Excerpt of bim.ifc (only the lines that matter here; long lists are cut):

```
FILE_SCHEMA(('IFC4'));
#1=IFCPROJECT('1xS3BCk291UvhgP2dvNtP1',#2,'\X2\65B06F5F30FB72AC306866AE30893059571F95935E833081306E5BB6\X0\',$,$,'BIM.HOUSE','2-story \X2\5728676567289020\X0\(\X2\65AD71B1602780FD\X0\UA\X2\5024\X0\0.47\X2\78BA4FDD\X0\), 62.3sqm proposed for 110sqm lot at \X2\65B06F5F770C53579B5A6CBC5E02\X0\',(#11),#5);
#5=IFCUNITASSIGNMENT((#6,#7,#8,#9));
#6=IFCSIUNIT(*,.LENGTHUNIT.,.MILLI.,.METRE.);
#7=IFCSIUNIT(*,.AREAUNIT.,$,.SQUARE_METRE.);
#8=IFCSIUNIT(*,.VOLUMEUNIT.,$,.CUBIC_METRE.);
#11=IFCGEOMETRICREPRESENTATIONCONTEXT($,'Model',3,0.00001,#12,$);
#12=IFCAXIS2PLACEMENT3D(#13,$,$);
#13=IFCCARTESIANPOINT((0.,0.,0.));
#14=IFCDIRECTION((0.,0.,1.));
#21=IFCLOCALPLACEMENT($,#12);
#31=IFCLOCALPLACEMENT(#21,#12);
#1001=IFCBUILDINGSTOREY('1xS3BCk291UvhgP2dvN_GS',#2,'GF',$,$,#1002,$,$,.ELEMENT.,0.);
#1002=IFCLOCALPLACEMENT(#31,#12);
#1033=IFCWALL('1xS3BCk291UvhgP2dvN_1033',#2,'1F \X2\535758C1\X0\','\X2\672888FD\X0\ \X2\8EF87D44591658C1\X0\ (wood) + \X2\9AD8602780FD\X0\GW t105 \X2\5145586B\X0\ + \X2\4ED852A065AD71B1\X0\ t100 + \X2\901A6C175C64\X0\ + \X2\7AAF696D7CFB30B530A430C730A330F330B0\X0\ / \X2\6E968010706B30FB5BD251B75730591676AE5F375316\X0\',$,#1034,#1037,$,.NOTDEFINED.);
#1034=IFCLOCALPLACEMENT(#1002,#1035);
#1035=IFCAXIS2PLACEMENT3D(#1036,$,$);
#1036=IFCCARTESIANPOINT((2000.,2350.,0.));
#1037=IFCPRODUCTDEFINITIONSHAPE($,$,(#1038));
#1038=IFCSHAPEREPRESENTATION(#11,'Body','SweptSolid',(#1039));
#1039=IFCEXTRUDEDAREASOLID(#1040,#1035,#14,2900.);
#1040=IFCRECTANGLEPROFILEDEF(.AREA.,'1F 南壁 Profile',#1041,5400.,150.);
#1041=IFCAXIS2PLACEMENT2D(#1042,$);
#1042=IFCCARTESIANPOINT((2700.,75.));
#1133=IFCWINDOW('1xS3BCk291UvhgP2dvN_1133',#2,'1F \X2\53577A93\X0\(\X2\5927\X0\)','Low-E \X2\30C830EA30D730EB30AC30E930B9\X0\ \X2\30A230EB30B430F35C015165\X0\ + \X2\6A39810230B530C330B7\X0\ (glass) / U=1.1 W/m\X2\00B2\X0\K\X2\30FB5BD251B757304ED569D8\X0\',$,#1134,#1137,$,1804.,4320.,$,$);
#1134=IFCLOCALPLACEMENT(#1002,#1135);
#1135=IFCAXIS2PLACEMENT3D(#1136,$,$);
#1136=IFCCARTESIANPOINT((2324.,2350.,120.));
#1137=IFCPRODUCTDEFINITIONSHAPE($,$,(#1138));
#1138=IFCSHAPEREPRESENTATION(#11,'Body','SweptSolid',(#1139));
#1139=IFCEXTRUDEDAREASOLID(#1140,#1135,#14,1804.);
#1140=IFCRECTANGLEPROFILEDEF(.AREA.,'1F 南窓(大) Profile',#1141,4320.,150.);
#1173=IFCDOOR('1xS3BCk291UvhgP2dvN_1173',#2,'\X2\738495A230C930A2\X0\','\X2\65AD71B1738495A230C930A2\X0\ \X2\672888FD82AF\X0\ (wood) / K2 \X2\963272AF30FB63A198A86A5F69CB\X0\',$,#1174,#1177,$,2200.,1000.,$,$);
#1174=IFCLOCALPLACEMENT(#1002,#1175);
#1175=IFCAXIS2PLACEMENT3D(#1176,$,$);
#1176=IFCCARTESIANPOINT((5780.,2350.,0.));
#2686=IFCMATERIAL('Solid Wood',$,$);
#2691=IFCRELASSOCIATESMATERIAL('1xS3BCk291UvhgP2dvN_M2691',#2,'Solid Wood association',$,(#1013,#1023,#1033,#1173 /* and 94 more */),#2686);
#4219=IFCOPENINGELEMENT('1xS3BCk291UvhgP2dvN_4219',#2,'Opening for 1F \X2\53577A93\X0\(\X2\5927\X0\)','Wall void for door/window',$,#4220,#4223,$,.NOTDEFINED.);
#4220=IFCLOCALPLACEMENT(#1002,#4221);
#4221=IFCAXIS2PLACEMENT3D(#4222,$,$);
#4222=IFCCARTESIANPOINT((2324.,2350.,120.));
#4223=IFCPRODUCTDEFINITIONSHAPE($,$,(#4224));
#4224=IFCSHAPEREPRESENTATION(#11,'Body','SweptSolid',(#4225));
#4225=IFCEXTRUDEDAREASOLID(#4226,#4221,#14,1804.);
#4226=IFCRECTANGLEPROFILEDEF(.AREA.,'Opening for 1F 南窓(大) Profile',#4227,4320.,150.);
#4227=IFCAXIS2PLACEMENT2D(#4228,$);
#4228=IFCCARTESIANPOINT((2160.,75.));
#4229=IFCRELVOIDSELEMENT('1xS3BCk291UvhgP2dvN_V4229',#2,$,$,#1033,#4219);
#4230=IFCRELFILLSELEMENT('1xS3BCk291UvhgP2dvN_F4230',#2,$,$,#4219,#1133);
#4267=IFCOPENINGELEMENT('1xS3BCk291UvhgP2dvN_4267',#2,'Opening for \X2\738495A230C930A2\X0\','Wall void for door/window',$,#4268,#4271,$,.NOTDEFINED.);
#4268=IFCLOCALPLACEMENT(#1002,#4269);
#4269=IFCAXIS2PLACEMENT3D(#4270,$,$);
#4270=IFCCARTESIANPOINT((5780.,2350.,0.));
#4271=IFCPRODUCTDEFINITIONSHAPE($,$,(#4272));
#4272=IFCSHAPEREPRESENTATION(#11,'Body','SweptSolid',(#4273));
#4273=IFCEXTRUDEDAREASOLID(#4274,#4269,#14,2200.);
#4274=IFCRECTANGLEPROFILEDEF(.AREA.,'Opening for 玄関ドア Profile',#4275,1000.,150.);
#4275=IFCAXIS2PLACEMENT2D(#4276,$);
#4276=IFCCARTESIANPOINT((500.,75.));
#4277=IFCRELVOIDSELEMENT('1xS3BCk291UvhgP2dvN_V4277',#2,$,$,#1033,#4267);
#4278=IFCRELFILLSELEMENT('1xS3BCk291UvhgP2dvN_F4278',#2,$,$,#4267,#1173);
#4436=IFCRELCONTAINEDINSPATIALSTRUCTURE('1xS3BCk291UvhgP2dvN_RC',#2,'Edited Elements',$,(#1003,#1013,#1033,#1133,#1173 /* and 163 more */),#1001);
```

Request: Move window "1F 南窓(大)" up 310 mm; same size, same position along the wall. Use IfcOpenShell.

```python
import numpy as np
import ifcopenshell
import ifcopenshell.api.geometry
import ifcopenshell.util.placement
import ifcopenshell.util.unit

model = ifcopenshell.open("bim.ifc")
unit_scale = ifcopenshell.util.unit.calculate_unit_scale(model)

window = model.by_guid("1xS3BCk291UvhgP2dvN_1133")
opening = window.FillsVoids[0].RelatingOpeningElement
dz = 310.0

shift = np.array([0.0, 0.0, dz])
# The window is not placed relative to its opening, so move both.
for product in (opening, window):
    matrix = ifcopenshell.util.placement.get_local_placement(product.ObjectPlacement)
    matrix[:3, 3] += shift
    ifcopenshell.api.geometry.edit_object_placement(model, product=product, matrix=matrix, is_si=False)

print(f"moved by {dz * unit_scale:+.3f} m")

model.write("bim_rev.ifc")
```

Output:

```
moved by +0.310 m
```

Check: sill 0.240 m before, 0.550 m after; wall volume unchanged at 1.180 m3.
